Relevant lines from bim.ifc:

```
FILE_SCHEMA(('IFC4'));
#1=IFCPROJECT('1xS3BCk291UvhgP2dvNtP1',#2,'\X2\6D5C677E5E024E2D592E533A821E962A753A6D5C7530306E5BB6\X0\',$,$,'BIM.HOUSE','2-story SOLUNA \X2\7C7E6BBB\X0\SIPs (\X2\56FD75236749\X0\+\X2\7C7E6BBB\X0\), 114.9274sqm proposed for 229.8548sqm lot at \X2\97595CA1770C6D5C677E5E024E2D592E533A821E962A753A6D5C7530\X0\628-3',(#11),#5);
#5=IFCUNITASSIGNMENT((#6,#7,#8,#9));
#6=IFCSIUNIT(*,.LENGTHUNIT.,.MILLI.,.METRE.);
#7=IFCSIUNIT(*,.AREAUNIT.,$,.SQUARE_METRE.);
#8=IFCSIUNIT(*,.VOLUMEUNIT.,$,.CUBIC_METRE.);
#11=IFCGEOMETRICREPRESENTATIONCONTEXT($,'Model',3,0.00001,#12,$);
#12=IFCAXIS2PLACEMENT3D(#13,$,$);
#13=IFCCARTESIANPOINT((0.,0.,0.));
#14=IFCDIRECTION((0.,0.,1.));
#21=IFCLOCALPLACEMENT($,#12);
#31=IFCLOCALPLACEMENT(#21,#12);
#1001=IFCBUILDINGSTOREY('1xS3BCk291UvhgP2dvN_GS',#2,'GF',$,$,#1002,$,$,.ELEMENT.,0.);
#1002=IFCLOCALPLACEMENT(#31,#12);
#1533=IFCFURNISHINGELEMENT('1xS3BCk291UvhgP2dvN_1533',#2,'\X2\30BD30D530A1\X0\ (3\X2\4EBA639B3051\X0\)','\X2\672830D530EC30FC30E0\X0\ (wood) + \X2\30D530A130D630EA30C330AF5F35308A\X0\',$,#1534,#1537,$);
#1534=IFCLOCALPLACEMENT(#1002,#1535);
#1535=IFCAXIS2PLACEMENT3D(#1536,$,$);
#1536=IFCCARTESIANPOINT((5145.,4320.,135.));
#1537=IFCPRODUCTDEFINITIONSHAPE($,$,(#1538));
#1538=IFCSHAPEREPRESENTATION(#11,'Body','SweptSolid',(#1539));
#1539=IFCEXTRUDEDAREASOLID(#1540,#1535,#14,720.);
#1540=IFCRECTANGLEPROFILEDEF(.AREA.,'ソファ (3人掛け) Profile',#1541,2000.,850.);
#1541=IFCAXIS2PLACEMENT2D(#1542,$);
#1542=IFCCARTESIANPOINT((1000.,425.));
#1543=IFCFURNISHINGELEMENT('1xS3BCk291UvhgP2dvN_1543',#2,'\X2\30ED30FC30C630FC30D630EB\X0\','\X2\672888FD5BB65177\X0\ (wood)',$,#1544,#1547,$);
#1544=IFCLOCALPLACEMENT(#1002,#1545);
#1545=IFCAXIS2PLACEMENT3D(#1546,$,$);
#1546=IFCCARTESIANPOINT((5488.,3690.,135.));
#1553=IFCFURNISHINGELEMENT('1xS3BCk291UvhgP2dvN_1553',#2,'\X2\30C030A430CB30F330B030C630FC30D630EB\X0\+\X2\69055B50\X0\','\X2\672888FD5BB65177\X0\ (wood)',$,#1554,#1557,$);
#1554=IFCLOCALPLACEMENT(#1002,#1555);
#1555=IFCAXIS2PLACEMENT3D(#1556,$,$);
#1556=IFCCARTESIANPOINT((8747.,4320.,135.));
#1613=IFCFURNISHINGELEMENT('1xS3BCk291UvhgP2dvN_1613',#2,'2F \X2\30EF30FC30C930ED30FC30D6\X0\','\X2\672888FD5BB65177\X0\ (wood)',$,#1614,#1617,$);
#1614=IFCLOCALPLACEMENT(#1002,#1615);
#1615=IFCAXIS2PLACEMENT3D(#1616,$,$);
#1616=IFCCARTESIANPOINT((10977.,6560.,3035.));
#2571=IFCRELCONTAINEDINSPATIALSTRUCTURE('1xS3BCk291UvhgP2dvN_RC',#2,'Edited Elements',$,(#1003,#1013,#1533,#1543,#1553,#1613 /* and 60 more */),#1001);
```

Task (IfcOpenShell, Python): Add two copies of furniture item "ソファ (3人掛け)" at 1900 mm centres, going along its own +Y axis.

```python
import ifcopenshell
import ifcopenshell.api.geometry
import ifcopenshell.api.root
import ifcopenshell.util.element
import ifcopenshell.util.placement
import ifcopenshell.util.unit

model = ifcopenshell.open("bim.ifc")
unit_scale = ifcopenshell.util.unit.calculate_unit_scale(model)


def reuse_history(source, copy):
    """copy_class also copies each property set's owner history, people and application; keep the originals."""
    for rel in copy.IsDefinedBy:
        if rel.is_a("IfcRelDefinesByProperties") and (history := rel.RelatingPropertyDefinition.OwnerHistory):
            rel.RelatingPropertyDefinition.OwnerHistory = source.OwnerHistory
            ifcopenshell.util.element.remove_deep2(model, history)


source = model.by_id(1533)
base = ifcopenshell.util.placement.get_local_placement(source.ObjectPlacement)
step = base[:3, 1] * 1.9 / unit_scale

for i in range(1, 3):
    copy = ifcopenshell.api.root.copy_class(model, product=source)
    copy.Representation = ifcopenshell.util.element.copy_deep(
        model, source.Representation, exclude=["IfcGeometricRepresentationContext", "IfcRepresentationMap"]
    )
    reuse_history(source, copy)
    matrix = base.copy()
    matrix[:3, 3] += i * step
    print("added at", matrix[:3, 3].round(3) + 0.0)
    ifcopenshell.api.geometry.edit_object_placement(model, product=copy, matrix=matrix, is_si=False)

model.write("bim_edited.ifc")
```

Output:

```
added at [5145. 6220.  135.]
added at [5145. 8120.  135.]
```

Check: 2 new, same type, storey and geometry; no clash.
